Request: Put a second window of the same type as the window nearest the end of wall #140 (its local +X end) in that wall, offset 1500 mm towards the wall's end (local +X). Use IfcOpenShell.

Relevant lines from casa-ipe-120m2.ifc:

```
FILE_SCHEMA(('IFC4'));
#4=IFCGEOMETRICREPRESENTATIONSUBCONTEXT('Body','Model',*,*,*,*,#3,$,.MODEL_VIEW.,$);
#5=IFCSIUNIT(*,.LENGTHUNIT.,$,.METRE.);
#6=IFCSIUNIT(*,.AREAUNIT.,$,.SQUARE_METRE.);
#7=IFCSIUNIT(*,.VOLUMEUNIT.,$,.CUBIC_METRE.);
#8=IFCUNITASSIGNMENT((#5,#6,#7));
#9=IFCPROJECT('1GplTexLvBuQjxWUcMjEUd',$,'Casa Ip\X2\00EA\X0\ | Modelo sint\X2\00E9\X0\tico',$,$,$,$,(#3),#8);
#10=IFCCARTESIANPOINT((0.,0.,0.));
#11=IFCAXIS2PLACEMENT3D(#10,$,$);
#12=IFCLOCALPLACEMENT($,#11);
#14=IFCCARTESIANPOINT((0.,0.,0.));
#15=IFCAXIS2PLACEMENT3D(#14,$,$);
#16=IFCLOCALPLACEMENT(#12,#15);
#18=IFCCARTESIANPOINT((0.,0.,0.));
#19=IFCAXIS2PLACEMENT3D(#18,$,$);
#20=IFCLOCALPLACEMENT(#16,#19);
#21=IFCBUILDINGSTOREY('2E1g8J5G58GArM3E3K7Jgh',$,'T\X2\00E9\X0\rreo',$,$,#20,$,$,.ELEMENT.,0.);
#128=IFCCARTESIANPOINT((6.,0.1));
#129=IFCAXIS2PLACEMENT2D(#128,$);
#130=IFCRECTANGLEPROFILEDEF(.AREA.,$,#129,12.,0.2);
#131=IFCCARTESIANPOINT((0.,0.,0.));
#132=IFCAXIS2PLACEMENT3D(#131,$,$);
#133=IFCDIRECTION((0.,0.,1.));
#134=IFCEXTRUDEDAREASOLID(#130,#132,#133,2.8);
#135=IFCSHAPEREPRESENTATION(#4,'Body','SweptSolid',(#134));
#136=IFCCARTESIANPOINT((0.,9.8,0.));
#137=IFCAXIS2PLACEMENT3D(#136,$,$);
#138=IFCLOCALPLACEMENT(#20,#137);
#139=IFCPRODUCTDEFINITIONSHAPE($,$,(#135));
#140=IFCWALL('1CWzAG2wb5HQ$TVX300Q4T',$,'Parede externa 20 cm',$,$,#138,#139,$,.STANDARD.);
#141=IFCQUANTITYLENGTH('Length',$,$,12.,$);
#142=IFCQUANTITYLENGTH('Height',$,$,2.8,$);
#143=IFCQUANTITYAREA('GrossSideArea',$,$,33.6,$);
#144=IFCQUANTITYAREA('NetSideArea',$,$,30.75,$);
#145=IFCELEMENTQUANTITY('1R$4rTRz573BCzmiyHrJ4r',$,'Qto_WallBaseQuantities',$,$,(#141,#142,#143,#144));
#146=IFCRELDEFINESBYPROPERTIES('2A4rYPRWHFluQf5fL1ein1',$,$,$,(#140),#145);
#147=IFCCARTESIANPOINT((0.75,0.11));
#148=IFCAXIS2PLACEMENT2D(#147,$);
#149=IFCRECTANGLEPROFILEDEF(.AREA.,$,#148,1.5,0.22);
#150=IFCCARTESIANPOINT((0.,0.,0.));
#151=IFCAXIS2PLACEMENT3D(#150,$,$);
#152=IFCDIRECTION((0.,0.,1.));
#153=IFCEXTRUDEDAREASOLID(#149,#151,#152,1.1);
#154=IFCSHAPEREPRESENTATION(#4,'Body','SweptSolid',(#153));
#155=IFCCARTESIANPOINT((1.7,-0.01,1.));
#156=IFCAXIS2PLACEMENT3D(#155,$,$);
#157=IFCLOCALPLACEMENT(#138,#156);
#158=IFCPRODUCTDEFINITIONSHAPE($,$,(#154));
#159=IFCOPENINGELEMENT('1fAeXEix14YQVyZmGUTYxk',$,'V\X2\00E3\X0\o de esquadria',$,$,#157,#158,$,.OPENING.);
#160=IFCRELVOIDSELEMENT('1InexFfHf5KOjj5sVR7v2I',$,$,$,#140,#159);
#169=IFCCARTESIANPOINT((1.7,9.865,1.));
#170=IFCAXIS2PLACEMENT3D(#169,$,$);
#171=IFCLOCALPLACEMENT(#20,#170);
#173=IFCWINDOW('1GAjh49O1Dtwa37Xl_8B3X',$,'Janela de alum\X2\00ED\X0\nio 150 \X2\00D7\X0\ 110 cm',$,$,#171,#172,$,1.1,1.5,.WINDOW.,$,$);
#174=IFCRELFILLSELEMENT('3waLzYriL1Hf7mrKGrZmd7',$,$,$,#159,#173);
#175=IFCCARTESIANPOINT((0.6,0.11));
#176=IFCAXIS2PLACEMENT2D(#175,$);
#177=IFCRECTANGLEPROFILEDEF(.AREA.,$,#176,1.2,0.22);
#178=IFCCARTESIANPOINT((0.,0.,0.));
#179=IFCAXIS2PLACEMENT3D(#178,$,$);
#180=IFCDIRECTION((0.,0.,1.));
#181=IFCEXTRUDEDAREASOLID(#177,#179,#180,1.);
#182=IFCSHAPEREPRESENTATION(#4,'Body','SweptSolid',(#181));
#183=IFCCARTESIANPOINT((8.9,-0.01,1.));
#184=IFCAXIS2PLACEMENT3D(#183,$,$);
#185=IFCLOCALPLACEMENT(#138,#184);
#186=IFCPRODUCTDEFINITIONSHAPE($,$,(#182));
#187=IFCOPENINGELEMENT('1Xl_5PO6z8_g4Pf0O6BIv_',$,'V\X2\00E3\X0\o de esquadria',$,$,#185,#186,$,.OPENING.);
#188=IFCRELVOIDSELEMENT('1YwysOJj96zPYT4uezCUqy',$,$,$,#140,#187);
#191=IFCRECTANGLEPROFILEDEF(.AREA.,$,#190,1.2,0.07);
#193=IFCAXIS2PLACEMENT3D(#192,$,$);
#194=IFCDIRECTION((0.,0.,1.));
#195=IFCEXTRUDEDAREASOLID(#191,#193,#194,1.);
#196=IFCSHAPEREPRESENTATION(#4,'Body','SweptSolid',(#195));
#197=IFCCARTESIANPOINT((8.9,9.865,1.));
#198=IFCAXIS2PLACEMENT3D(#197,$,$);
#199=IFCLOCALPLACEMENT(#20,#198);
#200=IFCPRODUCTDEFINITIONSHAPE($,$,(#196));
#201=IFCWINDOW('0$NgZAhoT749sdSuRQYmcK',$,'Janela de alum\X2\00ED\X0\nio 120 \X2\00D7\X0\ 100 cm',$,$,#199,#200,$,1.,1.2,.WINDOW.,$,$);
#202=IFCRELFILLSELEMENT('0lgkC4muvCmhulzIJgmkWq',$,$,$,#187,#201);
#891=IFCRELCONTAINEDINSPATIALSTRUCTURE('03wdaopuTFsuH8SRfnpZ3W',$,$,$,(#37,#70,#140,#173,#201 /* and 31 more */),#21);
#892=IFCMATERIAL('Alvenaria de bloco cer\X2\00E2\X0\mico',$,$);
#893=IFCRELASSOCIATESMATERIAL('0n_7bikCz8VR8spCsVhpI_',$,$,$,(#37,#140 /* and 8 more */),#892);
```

```python
import ifcopenshell
import ifcopenshell.api.feature
import ifcopenshell.api.geometry
import ifcopenshell.api.pset
import ifcopenshell.api.root
import ifcopenshell.geom
import ifcopenshell.util.element
import ifcopenshell.util.placement
import ifcopenshell.util.shape
import ifcopenshell.util.unit

model = ifcopenshell.open("casa-ipe-120m2.ifc")
unit_scale = ifcopenshell.util.unit.calculate_unit_scale(model)
area_scale = ifcopenshell.util.unit.calculate_unit_scale(model, "AREAUNIT")
settings = ifcopenshell.geom.settings()


def volume(element):
    """Net volume in cubic metres, openings subtracted."""
    shape = ifcopenshell.geom.create_shape(settings, element)
    return ifcopenshell.util.shape.get_volume(shape.geometry)


window = model.by_guid("0$NgZAhoT749sdSuRQYmcK")
opening = window.FillsVoids[0].RelatingOpeningElement
wall = opening.VoidsElements[0].RelatingBuildingElement
before = volume(wall)
shift = ifcopenshell.util.placement.get_local_placement(wall.ObjectPlacement)[:3, 0] * 1.5 / unit_scale

# copy_class copies the void relationship, type, container and properties, but no geometry.
new_opening = ifcopenshell.api.root.copy_class(model, product=opening)
new_opening.Representation = ifcopenshell.util.element.copy_deep(
    model, opening.Representation, exclude=["IfcGeometricRepresentationContext", "IfcRepresentationMap"]
)
new_window = ifcopenshell.api.root.copy_class(model, product=window)
new_window.Representation = ifcopenshell.util.element.copy_deep(
    model, window.Representation, exclude=["IfcGeometricRepresentationContext", "IfcRepresentationMap"]
)
ifcopenshell.api.feature.add_filling(model, opening=new_opening, element=new_window)

for old, new in ((opening, new_opening), (window, new_window)):
    matrix = ifcopenshell.util.placement.get_local_placement(old.ObjectPlacement)
    matrix[:3, 3] += shift
    ifcopenshell.api.geometry.edit_object_placement(model, product=new, matrix=matrix, is_si=False)

after = volume(wall)
thickness = 0.2  # wall thickness in metres

# Update the wall's stored quantities.
qto = model.by_id(ifcopenshell.util.element.get_pset(wall, "Qto_WallBaseQuantities", should_inherit=False)["id"])
ifcopenshell.api.pset.edit_qto(model, qto=qto, properties={"NetSideArea": after / thickness / area_scale})

print(f"wall volume {before:.3f} -> {after:.3f} m3")

model.write("casa-ipe-120m2_edited.ifc")
```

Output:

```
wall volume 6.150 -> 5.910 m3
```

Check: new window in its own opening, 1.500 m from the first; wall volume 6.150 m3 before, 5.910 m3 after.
